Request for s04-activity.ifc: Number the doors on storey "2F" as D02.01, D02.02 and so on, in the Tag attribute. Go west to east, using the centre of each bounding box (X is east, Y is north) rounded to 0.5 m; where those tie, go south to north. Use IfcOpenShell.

First a look at what the model holds.

```python
import ifcopenshell
import ifcopenshell.util.element
import ifcopenshell.util.placement

model = ifcopenshell.open("s04-activity.ifc")
print(model.schema)
storey = next(s for s in model.by_type("IfcBuildingStorey") if s.Name == "2F")
doors = [e for e in ifcopenshell.util.element.get_decomposition(storey) if e.is_a("IfcDoor")]
for e in sorted(doors, key=lambda e: e.id()):
    origin = ifcopenshell.util.placement.get_local_placement(e.ObjectPlacement)[:3, 3]
    print(e.id(), e.Tag, e.Name, origin.round(2) + 0.0, sep=" | ")
```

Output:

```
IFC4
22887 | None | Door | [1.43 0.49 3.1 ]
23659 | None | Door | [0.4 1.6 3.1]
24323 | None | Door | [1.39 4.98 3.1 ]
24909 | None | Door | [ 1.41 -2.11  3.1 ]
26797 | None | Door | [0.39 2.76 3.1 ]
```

```python
import ifcopenshell
import ifcopenshell.geom
import ifcopenshell.util.element
import ifcopenshell.util.shape

model = ifcopenshell.open("s04-activity.ifc")
settings = ifcopenshell.geom.settings()
settings.set("use-world-coords", True)


def centre(element):
    shape = ifcopenshell.geom.create_shape(settings, element)
    return ifcopenshell.util.shape.get_bbox_centroid(shape.geometry)


storey = next(s for s in model.by_type("IfcBuildingStorey") if s.Name == "2F")
doors = [e for e in ifcopenshell.util.element.get_decomposition(storey) if e.is_a("IfcDoor")]

# Insertion points can sit at a corner or the storey origin, so sort by the geometry (in metres).
centres = {e: centre(e) for e in doors}
doors.sort(key=lambda e: (round(centres[e][0] / 0.5), centres[e][1]))

for i, e in enumerate(doors, start=1):
    number = f"D02.{i:02d}"
    e.Tag = number
    print(e.id(), number)

model.write("s04-activity_v2.ifc")
```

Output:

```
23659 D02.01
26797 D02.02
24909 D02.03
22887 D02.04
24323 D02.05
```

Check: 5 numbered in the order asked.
